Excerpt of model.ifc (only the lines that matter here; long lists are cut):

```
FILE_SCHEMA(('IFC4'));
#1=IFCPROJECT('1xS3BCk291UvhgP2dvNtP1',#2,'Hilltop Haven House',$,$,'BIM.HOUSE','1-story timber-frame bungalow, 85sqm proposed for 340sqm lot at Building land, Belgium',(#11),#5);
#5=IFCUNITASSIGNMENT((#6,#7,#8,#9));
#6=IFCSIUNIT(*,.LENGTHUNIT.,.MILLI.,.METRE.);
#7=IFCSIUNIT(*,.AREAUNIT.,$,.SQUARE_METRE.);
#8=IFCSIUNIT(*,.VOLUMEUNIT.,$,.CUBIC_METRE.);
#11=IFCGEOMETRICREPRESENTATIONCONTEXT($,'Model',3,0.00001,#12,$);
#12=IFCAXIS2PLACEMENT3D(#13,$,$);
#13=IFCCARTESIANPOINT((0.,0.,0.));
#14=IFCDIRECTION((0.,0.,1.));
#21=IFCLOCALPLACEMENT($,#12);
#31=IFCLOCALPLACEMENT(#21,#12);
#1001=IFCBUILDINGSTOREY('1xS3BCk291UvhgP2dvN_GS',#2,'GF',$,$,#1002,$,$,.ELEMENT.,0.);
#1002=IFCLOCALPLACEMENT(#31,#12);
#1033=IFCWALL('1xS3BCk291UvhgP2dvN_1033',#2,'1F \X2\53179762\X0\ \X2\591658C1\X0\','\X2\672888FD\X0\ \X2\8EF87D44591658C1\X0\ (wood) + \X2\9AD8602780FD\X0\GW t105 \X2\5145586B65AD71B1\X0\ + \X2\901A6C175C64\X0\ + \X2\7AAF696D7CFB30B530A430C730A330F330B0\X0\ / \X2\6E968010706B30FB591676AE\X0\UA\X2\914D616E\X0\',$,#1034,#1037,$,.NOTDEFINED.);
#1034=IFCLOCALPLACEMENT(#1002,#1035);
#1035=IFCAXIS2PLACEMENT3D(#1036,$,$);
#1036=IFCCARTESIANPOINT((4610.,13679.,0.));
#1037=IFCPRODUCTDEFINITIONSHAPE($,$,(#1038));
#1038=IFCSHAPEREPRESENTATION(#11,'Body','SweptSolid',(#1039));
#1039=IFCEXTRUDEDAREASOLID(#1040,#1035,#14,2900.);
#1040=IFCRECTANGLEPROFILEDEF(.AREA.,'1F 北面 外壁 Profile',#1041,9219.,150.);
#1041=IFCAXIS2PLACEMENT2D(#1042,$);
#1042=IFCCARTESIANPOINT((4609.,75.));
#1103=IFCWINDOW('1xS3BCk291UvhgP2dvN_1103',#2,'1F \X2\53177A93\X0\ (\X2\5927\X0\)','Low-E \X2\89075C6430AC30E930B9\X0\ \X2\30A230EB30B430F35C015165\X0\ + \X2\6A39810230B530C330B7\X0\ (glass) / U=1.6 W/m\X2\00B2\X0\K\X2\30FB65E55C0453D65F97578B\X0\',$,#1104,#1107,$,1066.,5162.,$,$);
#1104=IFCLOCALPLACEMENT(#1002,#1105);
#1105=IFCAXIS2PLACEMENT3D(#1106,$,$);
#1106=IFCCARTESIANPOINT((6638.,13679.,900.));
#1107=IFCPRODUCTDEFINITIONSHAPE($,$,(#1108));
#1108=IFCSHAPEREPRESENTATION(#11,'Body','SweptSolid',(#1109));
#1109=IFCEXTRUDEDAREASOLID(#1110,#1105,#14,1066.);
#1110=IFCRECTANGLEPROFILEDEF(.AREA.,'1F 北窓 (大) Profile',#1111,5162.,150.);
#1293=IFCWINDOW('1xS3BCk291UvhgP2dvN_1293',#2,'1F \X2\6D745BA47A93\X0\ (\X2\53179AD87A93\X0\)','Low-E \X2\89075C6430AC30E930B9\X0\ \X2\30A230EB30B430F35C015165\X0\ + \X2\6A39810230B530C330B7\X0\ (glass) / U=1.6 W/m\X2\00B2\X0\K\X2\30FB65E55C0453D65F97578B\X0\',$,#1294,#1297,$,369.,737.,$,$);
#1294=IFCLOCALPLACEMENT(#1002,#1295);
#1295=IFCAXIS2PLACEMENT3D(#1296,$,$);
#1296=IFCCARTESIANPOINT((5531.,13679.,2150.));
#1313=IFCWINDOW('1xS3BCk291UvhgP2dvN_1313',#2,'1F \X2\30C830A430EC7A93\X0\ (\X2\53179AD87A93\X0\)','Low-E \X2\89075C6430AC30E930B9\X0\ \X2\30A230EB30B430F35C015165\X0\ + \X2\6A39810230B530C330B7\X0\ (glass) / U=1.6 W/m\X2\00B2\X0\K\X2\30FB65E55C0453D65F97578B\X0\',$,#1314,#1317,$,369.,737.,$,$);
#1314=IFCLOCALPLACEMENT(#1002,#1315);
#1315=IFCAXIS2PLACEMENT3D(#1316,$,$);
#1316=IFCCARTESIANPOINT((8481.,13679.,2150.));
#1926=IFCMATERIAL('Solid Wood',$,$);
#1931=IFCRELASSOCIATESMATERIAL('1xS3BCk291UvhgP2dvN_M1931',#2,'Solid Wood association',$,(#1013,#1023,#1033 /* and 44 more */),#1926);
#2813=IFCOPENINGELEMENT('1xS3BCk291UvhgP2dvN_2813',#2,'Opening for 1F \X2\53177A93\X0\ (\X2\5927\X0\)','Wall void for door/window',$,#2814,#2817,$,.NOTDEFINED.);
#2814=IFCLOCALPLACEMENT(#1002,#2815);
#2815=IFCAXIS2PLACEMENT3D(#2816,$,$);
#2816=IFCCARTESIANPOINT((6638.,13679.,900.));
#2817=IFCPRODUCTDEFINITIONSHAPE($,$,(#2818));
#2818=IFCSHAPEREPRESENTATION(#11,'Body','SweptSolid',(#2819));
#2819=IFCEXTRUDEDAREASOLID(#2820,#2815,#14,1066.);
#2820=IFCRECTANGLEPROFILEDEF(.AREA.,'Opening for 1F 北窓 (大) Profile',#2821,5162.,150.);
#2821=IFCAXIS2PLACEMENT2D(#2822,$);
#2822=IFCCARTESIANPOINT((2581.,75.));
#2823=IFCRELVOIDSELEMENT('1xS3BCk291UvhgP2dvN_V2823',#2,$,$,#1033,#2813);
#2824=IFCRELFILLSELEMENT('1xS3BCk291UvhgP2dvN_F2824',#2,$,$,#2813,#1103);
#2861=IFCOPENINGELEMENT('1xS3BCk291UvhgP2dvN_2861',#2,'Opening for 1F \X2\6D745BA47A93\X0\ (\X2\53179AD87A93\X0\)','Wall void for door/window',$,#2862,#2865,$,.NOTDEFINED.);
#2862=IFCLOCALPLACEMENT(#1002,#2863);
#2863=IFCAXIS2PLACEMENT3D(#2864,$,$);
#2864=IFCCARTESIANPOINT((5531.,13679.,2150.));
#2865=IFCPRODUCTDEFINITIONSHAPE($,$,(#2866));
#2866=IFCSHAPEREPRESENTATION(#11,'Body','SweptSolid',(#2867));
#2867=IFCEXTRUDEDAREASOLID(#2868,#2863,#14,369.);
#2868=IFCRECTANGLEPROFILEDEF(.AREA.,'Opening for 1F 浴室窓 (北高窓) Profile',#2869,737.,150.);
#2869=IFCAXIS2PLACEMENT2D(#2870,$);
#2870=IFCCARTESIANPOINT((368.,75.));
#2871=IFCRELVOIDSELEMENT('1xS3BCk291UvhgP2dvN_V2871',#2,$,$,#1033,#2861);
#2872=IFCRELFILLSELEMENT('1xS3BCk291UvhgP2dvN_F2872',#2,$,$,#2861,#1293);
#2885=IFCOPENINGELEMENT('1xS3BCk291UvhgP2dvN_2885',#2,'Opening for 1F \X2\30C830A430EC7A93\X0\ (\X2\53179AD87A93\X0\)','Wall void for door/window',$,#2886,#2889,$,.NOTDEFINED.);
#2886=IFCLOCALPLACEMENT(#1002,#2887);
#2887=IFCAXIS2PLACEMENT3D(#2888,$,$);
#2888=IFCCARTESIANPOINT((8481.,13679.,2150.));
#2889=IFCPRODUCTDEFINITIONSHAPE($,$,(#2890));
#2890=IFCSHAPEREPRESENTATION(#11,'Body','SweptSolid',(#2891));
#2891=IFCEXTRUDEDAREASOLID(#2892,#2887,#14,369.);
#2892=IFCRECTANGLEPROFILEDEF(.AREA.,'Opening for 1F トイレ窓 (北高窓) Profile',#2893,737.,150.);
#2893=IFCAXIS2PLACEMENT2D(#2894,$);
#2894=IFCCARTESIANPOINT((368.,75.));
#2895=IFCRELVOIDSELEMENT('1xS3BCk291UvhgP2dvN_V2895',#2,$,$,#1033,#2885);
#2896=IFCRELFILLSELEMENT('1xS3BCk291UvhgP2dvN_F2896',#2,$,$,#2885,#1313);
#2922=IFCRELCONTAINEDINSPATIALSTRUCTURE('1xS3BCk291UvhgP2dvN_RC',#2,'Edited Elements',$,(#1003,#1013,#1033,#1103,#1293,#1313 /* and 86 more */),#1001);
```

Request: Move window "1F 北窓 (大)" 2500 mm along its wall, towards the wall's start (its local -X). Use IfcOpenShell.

```python
import ifcopenshell
import ifcopenshell.api.geometry
import ifcopenshell.util.placement
import ifcopenshell.util.unit

model = ifcopenshell.open("model.ifc")
unit_scale = ifcopenshell.util.unit.calculate_unit_scale(model)

window = model.by_id(1103)
opening = window.FillsVoids[0].RelatingOpeningElement
wall = opening.VoidsElements[0].RelatingBuildingElement

wall_matrix = ifcopenshell.util.placement.get_local_placement(wall.ObjectPlacement)
shift = wall_matrix[:3, 0] * -2.5 / unit_scale
before = ifcopenshell.util.placement.get_local_placement(window.ObjectPlacement)[:3, 3].copy()

# The window is not placed relative to its opening, so move both.
for product in (opening, window):
    matrix = ifcopenshell.util.placement.get_local_placement(product.ObjectPlacement)
    matrix[:3, 3] += shift
    ifcopenshell.api.geometry.edit_object_placement(model, product=product, matrix=matrix, is_si=False)

after = ifcopenshell.util.placement.get_local_placement(window.ObjectPlacement)[:3, 3]
print("window moved by", (after - before).round(3) + 0.0)

model.write("model_rev.ifc")
```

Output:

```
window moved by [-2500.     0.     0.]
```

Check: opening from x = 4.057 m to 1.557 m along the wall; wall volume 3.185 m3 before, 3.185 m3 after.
